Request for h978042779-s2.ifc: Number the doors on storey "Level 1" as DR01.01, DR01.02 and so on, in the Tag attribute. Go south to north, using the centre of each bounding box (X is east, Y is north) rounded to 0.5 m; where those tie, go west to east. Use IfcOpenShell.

First a look at what the model holds.

```python
import ifcopenshell
import ifcopenshell.util.element
import ifcopenshell.util.placement

model = ifcopenshell.open("h978042779-s2.ifc")
print(model.schema)
storey = next(s for s in model.by_type("IfcBuildingStorey") if s.Name == "Level 1")
doors = [e for e in ifcopenshell.util.element.get_decomposition(storey) if e.is_a("IfcDoor")]
for e in sorted(doors, key=lambda e: e.id()):
    origin = ifcopenshell.util.placement.get_local_placement(e.ObjectPlacement)[:3, 3]
    print(e.id(), e.Tag, e.Name, origin.round(2) + 0.0, sep=" | ")
```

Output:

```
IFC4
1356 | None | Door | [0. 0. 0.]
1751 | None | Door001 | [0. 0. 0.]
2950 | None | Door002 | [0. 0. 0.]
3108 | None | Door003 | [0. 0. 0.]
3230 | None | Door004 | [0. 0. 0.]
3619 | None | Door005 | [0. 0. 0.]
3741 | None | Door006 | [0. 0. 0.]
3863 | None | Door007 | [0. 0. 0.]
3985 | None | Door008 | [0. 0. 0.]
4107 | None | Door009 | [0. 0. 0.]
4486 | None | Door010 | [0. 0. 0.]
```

```python
import ifcopenshell
import ifcopenshell.geom
import ifcopenshell.util.element
import ifcopenshell.util.shape

model = ifcopenshell.open("h978042779-s2.ifc")
settings = ifcopenshell.geom.settings()
settings.set("use-world-coords", True)


def centre(element):
    shape = ifcopenshell.geom.create_shape(settings, element)
    return ifcopenshell.util.shape.get_bbox_centroid(shape.geometry)


storey = next(s for s in model.by_type("IfcBuildingStorey") if s.Name == "Level 1")
doors = [e for e in ifcopenshell.util.element.get_decomposition(storey) if e.is_a("IfcDoor")]

# Insertion points can sit at a corner or the storey origin, so sort by the geometry (in metres).
centres = {e: centre(e) for e in doors}
doors.sort(key=lambda e: (round(centres[e][1] / 0.5), centres[e][0]))

for i, e in enumerate(doors, start=1):
    number = f"DR01.{i:02d}"
    e.Tag = number
    print(e.id(), number)

model.write("h978042779-s2_edited.ifc")
```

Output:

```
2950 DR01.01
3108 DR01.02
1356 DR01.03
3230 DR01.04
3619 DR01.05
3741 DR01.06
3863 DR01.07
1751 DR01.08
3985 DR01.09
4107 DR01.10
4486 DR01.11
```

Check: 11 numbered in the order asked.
